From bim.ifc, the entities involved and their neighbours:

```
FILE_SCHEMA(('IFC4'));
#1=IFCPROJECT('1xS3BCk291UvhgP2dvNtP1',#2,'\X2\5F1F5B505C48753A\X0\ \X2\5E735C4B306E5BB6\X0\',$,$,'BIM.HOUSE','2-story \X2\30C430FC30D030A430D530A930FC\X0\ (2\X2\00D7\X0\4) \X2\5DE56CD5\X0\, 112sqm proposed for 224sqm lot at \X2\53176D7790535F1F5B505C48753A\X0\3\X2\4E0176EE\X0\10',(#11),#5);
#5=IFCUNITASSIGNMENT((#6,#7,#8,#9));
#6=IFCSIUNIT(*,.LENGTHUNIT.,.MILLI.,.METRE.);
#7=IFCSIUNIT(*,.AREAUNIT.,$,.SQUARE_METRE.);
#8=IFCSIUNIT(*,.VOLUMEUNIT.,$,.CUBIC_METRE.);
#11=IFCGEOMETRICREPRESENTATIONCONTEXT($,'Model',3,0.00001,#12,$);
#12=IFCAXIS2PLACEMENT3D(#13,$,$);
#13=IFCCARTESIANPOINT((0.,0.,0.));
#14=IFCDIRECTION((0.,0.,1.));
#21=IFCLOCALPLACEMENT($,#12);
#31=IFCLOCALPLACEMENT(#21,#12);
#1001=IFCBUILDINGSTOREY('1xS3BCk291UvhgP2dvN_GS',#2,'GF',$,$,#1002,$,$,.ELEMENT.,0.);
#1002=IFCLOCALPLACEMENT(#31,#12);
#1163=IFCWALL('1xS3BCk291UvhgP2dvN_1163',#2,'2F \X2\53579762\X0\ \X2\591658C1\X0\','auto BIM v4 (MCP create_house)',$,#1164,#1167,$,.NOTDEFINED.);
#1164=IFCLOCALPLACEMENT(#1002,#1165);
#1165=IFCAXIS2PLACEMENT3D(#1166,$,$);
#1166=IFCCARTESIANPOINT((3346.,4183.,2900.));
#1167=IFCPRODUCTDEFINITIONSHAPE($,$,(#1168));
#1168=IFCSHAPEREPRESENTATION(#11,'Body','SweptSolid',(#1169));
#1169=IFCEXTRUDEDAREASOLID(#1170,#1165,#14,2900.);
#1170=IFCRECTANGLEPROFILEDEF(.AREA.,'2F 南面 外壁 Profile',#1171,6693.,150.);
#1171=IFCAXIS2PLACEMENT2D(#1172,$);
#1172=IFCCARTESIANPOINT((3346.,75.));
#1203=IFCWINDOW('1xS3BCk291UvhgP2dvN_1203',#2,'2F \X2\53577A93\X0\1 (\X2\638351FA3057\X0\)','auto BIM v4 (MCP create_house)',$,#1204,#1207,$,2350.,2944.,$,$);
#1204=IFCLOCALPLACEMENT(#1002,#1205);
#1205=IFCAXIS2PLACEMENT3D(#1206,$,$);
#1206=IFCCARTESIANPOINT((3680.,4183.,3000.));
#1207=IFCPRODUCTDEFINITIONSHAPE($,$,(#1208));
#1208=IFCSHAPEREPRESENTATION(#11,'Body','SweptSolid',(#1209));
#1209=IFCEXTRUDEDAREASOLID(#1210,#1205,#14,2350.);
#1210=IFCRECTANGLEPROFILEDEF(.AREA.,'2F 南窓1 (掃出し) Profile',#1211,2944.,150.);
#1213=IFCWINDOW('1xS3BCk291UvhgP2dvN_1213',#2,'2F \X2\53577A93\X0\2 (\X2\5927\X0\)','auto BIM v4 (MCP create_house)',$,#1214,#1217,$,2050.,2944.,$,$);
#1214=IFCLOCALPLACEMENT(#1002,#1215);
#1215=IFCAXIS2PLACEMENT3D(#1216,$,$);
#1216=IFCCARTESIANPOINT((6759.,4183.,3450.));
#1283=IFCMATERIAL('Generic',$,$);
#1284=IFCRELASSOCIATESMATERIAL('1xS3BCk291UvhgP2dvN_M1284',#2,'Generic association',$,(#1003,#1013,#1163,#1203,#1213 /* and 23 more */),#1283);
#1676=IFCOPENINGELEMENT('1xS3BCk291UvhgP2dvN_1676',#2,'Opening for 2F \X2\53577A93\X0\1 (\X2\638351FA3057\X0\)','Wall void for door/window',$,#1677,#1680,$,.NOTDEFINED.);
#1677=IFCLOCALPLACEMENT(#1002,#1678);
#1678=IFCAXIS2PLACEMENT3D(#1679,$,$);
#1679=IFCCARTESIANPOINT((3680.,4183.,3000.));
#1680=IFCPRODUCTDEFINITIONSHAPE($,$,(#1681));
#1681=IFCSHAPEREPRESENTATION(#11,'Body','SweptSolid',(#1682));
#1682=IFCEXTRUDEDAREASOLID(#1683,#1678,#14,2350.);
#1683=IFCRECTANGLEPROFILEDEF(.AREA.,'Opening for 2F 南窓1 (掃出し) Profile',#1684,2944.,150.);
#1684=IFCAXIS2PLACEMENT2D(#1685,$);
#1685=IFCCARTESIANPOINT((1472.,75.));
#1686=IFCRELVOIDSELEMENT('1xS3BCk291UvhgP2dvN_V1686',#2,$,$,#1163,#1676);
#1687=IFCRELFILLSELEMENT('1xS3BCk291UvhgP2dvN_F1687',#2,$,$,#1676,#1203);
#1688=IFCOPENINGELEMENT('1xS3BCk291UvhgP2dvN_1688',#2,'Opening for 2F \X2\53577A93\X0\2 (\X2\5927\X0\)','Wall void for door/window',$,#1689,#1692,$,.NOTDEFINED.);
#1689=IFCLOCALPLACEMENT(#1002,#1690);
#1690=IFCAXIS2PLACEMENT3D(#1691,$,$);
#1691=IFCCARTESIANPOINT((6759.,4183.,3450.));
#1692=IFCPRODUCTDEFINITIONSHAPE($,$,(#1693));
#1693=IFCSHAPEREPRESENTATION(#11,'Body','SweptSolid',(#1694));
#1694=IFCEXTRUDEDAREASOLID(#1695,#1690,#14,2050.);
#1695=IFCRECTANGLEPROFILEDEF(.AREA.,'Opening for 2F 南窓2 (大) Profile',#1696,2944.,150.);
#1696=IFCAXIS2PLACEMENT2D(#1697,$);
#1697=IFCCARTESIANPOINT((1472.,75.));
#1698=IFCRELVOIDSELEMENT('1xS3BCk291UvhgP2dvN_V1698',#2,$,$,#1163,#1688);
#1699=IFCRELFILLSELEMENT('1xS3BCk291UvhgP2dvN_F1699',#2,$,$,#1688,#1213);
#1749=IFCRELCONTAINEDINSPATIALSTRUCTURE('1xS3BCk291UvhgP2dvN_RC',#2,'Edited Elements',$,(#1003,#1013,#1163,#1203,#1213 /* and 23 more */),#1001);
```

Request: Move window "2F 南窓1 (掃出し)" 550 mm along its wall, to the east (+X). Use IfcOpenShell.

```python
import ifcopenshell
import ifcopenshell.api.geometry
import ifcopenshell.util.placement
import ifcopenshell.util.unit

model = ifcopenshell.open("bim.ifc")
unit_scale = ifcopenshell.util.unit.calculate_unit_scale(model)

window = model.by_id(1203)
opening = window.FillsVoids[0].RelatingOpeningElement
wall = opening.VoidsElements[0].RelatingBuildingElement

wall_matrix = ifcopenshell.util.placement.get_local_placement(wall.ObjectPlacement)
shift = wall_matrix[:3, 0] * 0.55 / unit_scale
before = ifcopenshell.util.placement.get_local_placement(window.ObjectPlacement)[:3, 3].copy()

# The window is not placed relative to its opening, so move both.
for product in (opening, window):
    matrix = ifcopenshell.util.placement.get_local_placement(product.ObjectPlacement)
    matrix[:3, 3] += shift
    ifcopenshell.api.geometry.edit_object_placement(model, product=product, matrix=matrix, is_si=False)

after = ifcopenshell.util.placement.get_local_placement(window.ObjectPlacement)[:3, 3]
print("window moved by", (after - before).round(3) + 0.0)

model.write("bim-out.ifc")
```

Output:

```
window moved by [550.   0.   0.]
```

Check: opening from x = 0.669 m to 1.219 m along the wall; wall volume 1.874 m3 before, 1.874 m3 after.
